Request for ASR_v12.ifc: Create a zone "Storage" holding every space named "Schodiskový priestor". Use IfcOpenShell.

First a look at what the model holds.

```python
import ifcopenshell

model = ifcopenshell.open("ASR_v12.ifc")
print(model.schema)
seen = {}
for space in model.by_type("IfcSpace"):
    seen[space.LongName] = seen.get(space.LongName, 0) + 1
for name, count in sorted(seen.items(), key=str):
    print(count, "x", name)
print("zones:", [z.Name for z in model.by_type("IfcZone")][:20])
```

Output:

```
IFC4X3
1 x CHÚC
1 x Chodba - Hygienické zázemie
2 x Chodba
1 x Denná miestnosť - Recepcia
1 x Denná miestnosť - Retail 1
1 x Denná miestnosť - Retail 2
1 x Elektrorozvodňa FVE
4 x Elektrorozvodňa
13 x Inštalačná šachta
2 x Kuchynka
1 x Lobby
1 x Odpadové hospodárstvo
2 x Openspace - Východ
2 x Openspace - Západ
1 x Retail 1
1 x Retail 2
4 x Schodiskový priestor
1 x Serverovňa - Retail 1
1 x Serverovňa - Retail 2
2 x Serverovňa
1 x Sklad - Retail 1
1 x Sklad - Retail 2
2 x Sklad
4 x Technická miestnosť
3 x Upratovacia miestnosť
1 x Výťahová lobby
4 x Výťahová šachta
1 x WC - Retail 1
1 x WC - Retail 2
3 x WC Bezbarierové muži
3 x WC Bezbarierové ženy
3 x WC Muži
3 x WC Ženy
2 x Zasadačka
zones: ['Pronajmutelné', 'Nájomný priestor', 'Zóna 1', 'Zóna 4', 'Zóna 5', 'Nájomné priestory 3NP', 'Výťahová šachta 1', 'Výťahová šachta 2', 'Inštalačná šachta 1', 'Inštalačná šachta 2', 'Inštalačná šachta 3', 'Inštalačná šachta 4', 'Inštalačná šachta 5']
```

```python
import ifcopenshell
import ifcopenshell.api.group
import ifcopenshell.api.root

model = ifcopenshell.open("ASR_v12.ifc")

names = {"Schodiskový priestor"}
spaces = [s for s in model.by_type("IfcSpace") if s.LongName in names]

zone = ifcopenshell.api.root.create_entity(model, ifc_class="IfcZone", name="Storage")
ifcopenshell.api.group.assign_group(model, products=spaces, group=zone)
print(len(spaces), "spaces in", zone.Name)

model.write("ASR_v12-out.ifc")
```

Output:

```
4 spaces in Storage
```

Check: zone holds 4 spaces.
